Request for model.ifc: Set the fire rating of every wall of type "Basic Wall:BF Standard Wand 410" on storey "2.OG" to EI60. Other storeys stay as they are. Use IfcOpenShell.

First a look at what the model holds.

```python
import ifcopenshell
import ifcopenshell.util.element

model = ifcopenshell.open("model.ifc")
print(model.schema)
storey = next(s for s in model.by_type("IfcBuildingStorey") if s.Name == "2.OG")
walls = [e for e in ifcopenshell.util.element.get_decomposition(storey) if e.is_a("IfcWall")]
seen = {}
for e in walls:
    element_type = ifcopenshell.util.element.get_type(e)
    key = (element_type.Name if element_type != e and element_type else None, ifcopenshell.util.element.get_pset(e, "Pset_WallCommon", "FireRating"))
    seen[key] = seen.get(key, 0) + 1
for (name, value), count in sorted(seen.items(), key=str):
    print(count, "x", name, "|", value)
```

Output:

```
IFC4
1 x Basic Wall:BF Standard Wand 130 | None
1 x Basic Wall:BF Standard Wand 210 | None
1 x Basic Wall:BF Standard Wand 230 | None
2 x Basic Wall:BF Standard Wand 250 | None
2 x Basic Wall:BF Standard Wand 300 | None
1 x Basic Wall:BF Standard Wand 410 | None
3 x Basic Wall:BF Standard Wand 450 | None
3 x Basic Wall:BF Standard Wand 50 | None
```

```python
import ifcopenshell
import ifcopenshell.api.pset
import ifcopenshell.util.element

model = ifcopenshell.open("model.ifc")

storey = next(s for s in model.by_type("IfcBuildingStorey") if s.Name == "2.OG")
walls = [e for e in ifcopenshell.util.element.get_decomposition(storey) if e.is_a("IfcWall")]

count = 0
for e in walls:
    element_type = ifcopenshell.util.element.get_type(e)
    if element_type in (None, e) or element_type.Name != "Basic Wall:BF Standard Wand 410":
        continue
    # add_pset returns the element's existing set when there is one.
    pset = ifcopenshell.api.pset.add_pset(model, product=e, name="Pset_WallCommon")
    ifcopenshell.api.pset.edit_pset(model, pset=pset, properties={"FireRating": "EI60"})
    count += 1

print(count, "walls updated")

model.write("model_rev.ifc")
```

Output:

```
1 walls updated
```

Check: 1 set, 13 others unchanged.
